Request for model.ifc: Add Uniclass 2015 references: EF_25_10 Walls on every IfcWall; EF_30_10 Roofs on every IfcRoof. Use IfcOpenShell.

First a look at what the model holds.

```python
import ifcopenshell

model = ifcopenshell.open("model.ifc")
print(model.schema)
print("classifications:", [c.Name for c in model.by_type("IfcClassification")])
for ifc_class in ("IfcDoor", "IfcRoof", "IfcStair", "IfcWall", "IfcWindow"):
    print(ifc_class, len(model.by_type(ifc_class)))
```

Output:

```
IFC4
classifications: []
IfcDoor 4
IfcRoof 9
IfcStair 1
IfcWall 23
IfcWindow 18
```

```python
import ifcopenshell
import ifcopenshell.api.classification

model = ifcopenshell.open("model.ifc")

system = ifcopenshell.api.classification.add_classification(model, classification="Uniclass 2015")

codes = {
    "IfcWall": ("EF_25_10", "Walls"),
    "IfcRoof": ("EF_30_10", "Roofs"),
}
for ifc_class, (code, name) in codes.items():
    products = model.by_type(ifc_class)
    ifcopenshell.api.classification.add_reference(
        model, products=products, classification=system, identification=code, name=name
    )
    print(code, len(products))

model.write("model_edited.ifc")
```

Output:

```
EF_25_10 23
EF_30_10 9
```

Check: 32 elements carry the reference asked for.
